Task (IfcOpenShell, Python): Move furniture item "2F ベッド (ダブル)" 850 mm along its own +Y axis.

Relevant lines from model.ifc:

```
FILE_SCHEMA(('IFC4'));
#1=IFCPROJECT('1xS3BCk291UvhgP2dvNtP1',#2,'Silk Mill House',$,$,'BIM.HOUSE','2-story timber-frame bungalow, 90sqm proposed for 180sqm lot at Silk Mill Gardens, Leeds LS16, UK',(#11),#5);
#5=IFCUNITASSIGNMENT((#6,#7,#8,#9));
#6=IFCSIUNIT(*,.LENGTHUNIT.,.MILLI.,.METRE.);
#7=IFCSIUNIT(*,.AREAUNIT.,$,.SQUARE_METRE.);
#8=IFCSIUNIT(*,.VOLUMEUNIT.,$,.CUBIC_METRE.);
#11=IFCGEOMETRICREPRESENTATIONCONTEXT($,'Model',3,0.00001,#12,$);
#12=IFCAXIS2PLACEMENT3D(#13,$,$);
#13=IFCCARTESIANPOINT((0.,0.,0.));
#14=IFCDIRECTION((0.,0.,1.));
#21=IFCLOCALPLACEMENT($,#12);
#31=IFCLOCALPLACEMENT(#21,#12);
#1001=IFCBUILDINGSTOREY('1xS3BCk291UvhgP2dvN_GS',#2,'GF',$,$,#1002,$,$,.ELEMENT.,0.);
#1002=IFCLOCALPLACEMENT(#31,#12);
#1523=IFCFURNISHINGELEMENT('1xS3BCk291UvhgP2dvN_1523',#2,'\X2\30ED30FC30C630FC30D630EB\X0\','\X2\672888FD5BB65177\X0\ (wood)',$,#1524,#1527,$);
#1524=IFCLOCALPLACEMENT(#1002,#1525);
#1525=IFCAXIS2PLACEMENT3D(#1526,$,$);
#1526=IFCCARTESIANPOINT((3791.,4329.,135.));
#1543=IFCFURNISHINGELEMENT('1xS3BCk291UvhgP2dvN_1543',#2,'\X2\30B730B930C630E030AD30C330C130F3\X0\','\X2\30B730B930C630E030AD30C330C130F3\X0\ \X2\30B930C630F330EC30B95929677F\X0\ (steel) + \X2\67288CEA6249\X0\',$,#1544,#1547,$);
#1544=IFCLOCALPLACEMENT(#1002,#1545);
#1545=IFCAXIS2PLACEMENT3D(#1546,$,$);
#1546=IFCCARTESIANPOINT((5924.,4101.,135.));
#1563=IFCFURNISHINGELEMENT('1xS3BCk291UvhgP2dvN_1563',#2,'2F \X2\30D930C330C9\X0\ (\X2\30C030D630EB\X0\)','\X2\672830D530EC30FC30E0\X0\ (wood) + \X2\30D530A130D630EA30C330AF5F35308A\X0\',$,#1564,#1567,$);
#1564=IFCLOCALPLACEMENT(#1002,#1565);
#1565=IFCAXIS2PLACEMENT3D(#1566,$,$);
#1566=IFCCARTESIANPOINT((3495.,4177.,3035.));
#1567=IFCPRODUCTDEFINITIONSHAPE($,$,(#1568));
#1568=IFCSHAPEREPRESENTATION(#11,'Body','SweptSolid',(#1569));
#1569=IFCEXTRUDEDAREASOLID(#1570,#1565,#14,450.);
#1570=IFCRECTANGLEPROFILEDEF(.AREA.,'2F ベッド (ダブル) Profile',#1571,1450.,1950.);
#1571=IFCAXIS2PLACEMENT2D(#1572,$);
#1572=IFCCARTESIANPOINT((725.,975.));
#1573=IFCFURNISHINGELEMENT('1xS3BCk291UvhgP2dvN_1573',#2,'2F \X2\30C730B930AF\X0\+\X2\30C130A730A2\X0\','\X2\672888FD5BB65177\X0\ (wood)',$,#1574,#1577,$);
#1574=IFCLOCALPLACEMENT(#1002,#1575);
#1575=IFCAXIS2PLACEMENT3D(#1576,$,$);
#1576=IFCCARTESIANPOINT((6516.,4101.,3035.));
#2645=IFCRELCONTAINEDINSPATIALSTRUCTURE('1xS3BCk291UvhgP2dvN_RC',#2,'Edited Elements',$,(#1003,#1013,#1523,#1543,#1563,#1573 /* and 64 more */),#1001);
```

```python
import ifcopenshell
import ifcopenshell.api.geometry
import ifcopenshell.util.placement

model = ifcopenshell.open("model.ifc")

item = model.by_id(1563)
matrix = ifcopenshell.util.placement.get_local_placement(item.ObjectPlacement)
matrix[:3, 3] += matrix[:3, 1] * 850.0
ifcopenshell.api.geometry.edit_object_placement(model, product=item, matrix=matrix, is_si=False)

print(ifcopenshell.util.placement.get_local_placement(item.ObjectPlacement).round(3) + 0.0)

model.write("model_v2.ifc")
```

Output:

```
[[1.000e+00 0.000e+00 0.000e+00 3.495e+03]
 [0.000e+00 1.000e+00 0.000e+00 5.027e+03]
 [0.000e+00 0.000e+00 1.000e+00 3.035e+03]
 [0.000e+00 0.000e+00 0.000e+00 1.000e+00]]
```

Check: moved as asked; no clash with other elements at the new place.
